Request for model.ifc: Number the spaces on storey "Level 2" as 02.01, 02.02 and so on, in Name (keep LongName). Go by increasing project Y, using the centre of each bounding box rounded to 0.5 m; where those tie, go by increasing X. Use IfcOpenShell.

First a look at what the model holds.

```python
import ifcopenshell
import ifcopenshell.util.element
import ifcopenshell.util.placement

model = ifcopenshell.open("model.ifc")
print(model.schema)
storey = next(s for s in model.by_type("IfcBuildingStorey") if s.Name == "Level 2")
spaces = [e for e in ifcopenshell.util.element.get_decomposition(storey) if e.is_a("IfcSpace")]
for e in sorted(spaces, key=lambda e: e.id()):
    origin = ifcopenshell.util.placement.get_local_placement(e.ObjectPlacement)[:3, 3]
    print(e.id(), e.Name, e.LongName, origin.round(2) + 0.0, sep=" | ")
```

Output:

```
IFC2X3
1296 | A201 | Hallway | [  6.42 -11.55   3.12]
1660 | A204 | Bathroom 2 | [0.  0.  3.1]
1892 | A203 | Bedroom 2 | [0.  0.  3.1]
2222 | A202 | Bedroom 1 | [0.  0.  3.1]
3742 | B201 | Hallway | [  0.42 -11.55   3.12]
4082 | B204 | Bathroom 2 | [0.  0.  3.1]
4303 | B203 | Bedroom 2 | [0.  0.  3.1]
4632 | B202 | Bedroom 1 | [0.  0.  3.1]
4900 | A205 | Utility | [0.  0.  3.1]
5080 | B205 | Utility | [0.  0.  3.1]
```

```python
import ifcopenshell
import ifcopenshell.geom
import ifcopenshell.util.element
import ifcopenshell.util.shape

model = ifcopenshell.open("model.ifc")
settings = ifcopenshell.geom.settings()
settings.set("use-world-coords", True)


def centre(element):
    shape = ifcopenshell.geom.create_shape(settings, element)
    return ifcopenshell.util.shape.get_bbox_centroid(shape.geometry)


storey = next(s for s in model.by_type("IfcBuildingStorey") if s.Name == "Level 2")
spaces = [e for e in ifcopenshell.util.element.get_decomposition(storey) if e.is_a("IfcSpace")]

# Insertion points can sit at a corner or the storey origin, so sort by the geometry (in metres).
centres = {e: centre(e) for e in spaces}
spaces.sort(key=lambda e: (round(centres[e][1] / 0.5), centres[e][0]))

for i, e in enumerate(spaces, start=1):
    number = f"02.{i:02d}"
    e.Name = number
    print(e.id(), number)

model.write("model_v2.ifc")
```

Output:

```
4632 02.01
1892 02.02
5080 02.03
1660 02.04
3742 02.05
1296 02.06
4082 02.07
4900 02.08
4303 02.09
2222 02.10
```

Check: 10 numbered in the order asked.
